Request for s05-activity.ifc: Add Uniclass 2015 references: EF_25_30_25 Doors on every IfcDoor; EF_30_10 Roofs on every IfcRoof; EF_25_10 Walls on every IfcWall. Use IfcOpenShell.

First a look at what the model holds.

```python
import ifcopenshell

model = ifcopenshell.open("s05-activity.ifc")
print(model.schema)
print("classifications:", [c.Name for c in model.by_type("IfcClassification")])
for ifc_class in ("IfcDoor", "IfcRoof", "IfcStair", "IfcWall", "IfcWindow"):
    print(ifc_class, len(model.by_type(ifc_class)))
```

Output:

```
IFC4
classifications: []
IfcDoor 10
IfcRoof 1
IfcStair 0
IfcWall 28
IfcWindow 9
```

```python
import ifcopenshell
import ifcopenshell.api.classification

model = ifcopenshell.open("s05-activity.ifc")

system = ifcopenshell.api.classification.add_classification(model, classification="Uniclass 2015")

codes = {
    "IfcDoor": ("EF_25_30_25", "Doors"),
    "IfcRoof": ("EF_30_10", "Roofs"),
    "IfcWall": ("EF_25_10", "Walls"),
}
for ifc_class, (code, name) in codes.items():
    products = model.by_type(ifc_class)
    ifcopenshell.api.classification.add_reference(
        model, products=products, classification=system, identification=code, name=name
    )
    print(code, len(products))

model.write("s05-activity-out.ifc")
```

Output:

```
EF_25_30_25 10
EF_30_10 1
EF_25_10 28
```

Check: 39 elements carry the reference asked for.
